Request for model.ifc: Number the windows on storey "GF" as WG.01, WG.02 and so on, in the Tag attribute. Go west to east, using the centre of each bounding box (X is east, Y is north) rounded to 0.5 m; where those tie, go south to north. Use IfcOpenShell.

First a look at what the model holds.

```python
import ifcopenshell
import ifcopenshell.util.element
import ifcopenshell.util.placement

model = ifcopenshell.open("model.ifc")
print(model.schema)
storey = next(s for s in model.by_type("IfcBuildingStorey") if s.Name == "GF")
windows = [e for e in ifcopenshell.util.element.get_decomposition(storey) if e.is_a("IfcWindow")]
for e in sorted(windows, key=lambda e: e.id()):
    origin = ifcopenshell.util.placement.get_local_placement(e.ObjectPlacement)[:3, 3]
    print(e.id(), e.Tag, e.Name, origin.round(2) + 0.0, sep=" | ")
```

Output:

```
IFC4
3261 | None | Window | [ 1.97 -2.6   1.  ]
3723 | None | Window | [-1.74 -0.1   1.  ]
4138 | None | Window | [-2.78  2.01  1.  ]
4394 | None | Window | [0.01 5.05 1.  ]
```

```python
import ifcopenshell
import ifcopenshell.geom
import ifcopenshell.util.element
import ifcopenshell.util.shape

model = ifcopenshell.open("model.ifc")
settings = ifcopenshell.geom.settings()
settings.set("use-world-coords", True)


def centre(element):
    shape = ifcopenshell.geom.create_shape(settings, element)
    return ifcopenshell.util.shape.get_bbox_centroid(shape.geometry)


storey = next(s for s in model.by_type("IfcBuildingStorey") if s.Name == "GF")
windows = [e for e in ifcopenshell.util.element.get_decomposition(storey) if e.is_a("IfcWindow")]

# Insertion points can sit at a corner or the storey origin, so sort by the geometry (in metres).
centres = {e: centre(e) for e in windows}
windows.sort(key=lambda e: (round(centres[e][0] / 0.5), centres[e][1]))

for i, e in enumerate(windows, start=1):
    number = f"WG.{i:02d}"
    e.Tag = number
    print(e.id(), number)

model.write("model_rev.ifc")
```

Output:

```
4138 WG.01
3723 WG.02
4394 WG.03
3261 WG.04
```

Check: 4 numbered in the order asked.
